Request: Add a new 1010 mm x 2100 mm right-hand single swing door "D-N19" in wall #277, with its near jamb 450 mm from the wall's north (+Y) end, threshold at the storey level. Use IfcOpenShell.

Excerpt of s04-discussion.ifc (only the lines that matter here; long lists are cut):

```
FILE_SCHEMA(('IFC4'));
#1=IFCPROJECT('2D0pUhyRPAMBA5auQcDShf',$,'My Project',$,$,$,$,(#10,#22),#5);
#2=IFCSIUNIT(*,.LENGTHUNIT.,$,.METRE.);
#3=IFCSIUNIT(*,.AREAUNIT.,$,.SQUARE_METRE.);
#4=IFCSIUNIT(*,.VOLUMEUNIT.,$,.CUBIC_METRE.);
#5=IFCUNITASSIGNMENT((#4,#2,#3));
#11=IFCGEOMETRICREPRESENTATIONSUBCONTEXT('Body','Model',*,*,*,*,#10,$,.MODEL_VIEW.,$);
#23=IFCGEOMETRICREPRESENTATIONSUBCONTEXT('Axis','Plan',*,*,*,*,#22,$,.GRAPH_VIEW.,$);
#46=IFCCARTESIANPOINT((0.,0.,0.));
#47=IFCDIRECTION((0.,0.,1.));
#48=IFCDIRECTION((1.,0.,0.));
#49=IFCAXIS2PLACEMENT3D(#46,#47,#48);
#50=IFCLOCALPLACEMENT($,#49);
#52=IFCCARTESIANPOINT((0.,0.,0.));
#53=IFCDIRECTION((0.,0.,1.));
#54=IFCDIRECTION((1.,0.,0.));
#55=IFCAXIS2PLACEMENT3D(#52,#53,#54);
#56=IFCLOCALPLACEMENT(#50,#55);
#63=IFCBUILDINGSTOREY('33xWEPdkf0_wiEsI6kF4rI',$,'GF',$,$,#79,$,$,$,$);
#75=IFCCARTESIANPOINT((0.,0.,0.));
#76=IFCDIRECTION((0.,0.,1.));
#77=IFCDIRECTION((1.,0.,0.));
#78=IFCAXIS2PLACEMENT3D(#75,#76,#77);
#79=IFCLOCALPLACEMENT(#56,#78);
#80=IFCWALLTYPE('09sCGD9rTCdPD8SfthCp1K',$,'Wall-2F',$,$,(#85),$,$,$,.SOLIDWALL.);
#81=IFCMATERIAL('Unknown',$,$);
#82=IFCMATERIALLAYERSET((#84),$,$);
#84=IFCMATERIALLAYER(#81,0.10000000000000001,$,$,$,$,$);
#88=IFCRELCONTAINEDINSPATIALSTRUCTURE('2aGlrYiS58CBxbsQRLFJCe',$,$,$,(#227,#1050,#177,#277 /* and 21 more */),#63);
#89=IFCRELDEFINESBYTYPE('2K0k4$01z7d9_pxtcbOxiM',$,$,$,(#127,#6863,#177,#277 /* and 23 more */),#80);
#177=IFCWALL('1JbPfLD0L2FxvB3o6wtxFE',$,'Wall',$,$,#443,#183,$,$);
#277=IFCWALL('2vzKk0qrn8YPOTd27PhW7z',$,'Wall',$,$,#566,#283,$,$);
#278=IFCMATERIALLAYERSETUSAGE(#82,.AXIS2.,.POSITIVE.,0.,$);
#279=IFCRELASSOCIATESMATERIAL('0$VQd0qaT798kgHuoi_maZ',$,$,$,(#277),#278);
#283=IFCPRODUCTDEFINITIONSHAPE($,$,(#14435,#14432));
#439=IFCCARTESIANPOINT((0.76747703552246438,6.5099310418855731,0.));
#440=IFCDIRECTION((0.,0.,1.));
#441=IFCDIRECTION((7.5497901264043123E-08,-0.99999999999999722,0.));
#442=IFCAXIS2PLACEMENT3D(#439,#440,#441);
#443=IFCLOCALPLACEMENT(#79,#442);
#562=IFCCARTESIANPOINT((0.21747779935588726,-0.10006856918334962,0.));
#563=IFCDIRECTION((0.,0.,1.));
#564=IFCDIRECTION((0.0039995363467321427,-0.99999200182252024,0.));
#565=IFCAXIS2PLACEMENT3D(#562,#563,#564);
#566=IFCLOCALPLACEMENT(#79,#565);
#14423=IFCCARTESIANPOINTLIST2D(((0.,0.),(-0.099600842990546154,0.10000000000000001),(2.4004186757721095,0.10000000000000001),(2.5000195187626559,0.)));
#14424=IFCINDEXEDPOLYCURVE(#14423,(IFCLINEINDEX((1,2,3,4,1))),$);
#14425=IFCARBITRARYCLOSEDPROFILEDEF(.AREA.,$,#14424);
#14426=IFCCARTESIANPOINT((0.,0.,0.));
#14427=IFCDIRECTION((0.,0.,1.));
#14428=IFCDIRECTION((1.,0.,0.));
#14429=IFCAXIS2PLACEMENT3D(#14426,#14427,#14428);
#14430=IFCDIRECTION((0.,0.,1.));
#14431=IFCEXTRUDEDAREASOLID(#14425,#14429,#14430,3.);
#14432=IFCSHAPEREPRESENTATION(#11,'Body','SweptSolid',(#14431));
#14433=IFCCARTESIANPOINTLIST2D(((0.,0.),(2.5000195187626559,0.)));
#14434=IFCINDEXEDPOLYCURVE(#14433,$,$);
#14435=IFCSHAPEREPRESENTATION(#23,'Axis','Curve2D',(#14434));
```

```python
import numpy as np
import ifcopenshell
import ifcopenshell.api.feature
import ifcopenshell.api.geometry
import ifcopenshell.api.root
import ifcopenshell.api.spatial
import ifcopenshell.geom
import ifcopenshell.util.element
import ifcopenshell.util.placement
import ifcopenshell.util.representation
import ifcopenshell.util.shape
import ifcopenshell.util.unit

model = ifcopenshell.open("s04-discussion.ifc")
unit_scale = ifcopenshell.util.unit.calculate_unit_scale(model)
settings = ifcopenshell.geom.settings()


def volume(element):
    """Net volume in cubic metres, openings subtracted."""
    shape = ifcopenshell.geom.create_shape(settings, element)
    return ifcopenshell.util.shape.get_volume(shape.geometry)


wall = model.by_guid("2vzKk0qrn8YPOTd27PhW7z")
storey = ifcopenshell.util.element.get_container(wall, ifc_class="IfcBuildingStorey")
context = ifcopenshell.util.representation.get_context(model, "Model", "Body", "MODEL_VIEW")
before = volume(wall)

width, height, from_end, sill = 1.01, 2.1, 0.45, 0.0  # metres

# The wall runs along its own X axis, and the end named is its -X end.
wall_shape = ifcopenshell.geom.create_shape(settings, wall)
x, y, z = ifcopenshell.util.shape.get_vertices(wall_shape.geometry).T
start = x.min() + from_end
face, thickness = float(y.min()), float(y.max() - y.min())
wall_matrix = ifcopenshell.util.placement.get_local_placement(wall.ObjectPlacement)
level = ifcopenshell.util.placement.get_local_placement(storey.ObjectPlacement)[2, 3]


def in_wall(x, y):
    """Placement at x, y metres in the wall's axes, at sill height."""
    matrix = wall_matrix.copy()
    matrix[:, 3] = wall_matrix @ np.array([x / unit_scale, y / unit_scale, 0.0, 1.0])
    matrix[2, 3] = level + sill / unit_scale
    return matrix


# Opening: a box that overshoots both wall faces by 50 mm.
opening = ifcopenshell.api.root.create_entity(model, ifc_class="IfcOpeningElement", predefined_type="OPENING")
box = ifcopenshell.api.geometry.add_wall_representation(
    model, context=context, length=width, height=height, thickness=thickness + 0.1
)
ifcopenshell.api.geometry.assign_representation(model, product=opening, representation=box)
ifcopenshell.api.geometry.edit_object_placement(model, product=opening, matrix=in_wall(start, face - 0.05), is_si=False)
ifcopenshell.api.feature.add_feature(model, feature=opening, element=wall)

door = ifcopenshell.api.root.create_entity(model, ifc_class="IfcDoor", name="D-N19", predefined_type="DOOR")
door.OverallWidth, door.OverallHeight = width / unit_scale, height / unit_scale
door.OperationType = "SINGLE_SWING_RIGHT"
body = ifcopenshell.api.geometry.add_door_representation(
    model,
    context=context,
    overall_width=door.OverallWidth,
    overall_height=door.OverallHeight,
    operation_type="SINGLE_SWING_RIGHT",
    lining_properties={"LiningDepth": thickness / unit_scale, "ThresholdDepth": thickness / unit_scale},
)
ifcopenshell.api.geometry.assign_representation(model, product=door, representation=body)
ifcopenshell.api.spatial.assign_container(model, products=[door], relating_structure=storey)
ifcopenshell.api.feature.add_filling(model, opening=opening, element=door)

# The lining spans the wall, so the door starts at the wall face.
ifcopenshell.api.geometry.edit_object_placement(model, product=door, matrix=in_wall(start, face), is_si=False)

after = volume(wall)

print(f"wall volume {before:.3f} -> {after:.3f} m3")

model.write("s04-discussion_rev.ifc")
```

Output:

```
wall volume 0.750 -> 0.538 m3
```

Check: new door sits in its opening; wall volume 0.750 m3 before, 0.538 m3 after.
